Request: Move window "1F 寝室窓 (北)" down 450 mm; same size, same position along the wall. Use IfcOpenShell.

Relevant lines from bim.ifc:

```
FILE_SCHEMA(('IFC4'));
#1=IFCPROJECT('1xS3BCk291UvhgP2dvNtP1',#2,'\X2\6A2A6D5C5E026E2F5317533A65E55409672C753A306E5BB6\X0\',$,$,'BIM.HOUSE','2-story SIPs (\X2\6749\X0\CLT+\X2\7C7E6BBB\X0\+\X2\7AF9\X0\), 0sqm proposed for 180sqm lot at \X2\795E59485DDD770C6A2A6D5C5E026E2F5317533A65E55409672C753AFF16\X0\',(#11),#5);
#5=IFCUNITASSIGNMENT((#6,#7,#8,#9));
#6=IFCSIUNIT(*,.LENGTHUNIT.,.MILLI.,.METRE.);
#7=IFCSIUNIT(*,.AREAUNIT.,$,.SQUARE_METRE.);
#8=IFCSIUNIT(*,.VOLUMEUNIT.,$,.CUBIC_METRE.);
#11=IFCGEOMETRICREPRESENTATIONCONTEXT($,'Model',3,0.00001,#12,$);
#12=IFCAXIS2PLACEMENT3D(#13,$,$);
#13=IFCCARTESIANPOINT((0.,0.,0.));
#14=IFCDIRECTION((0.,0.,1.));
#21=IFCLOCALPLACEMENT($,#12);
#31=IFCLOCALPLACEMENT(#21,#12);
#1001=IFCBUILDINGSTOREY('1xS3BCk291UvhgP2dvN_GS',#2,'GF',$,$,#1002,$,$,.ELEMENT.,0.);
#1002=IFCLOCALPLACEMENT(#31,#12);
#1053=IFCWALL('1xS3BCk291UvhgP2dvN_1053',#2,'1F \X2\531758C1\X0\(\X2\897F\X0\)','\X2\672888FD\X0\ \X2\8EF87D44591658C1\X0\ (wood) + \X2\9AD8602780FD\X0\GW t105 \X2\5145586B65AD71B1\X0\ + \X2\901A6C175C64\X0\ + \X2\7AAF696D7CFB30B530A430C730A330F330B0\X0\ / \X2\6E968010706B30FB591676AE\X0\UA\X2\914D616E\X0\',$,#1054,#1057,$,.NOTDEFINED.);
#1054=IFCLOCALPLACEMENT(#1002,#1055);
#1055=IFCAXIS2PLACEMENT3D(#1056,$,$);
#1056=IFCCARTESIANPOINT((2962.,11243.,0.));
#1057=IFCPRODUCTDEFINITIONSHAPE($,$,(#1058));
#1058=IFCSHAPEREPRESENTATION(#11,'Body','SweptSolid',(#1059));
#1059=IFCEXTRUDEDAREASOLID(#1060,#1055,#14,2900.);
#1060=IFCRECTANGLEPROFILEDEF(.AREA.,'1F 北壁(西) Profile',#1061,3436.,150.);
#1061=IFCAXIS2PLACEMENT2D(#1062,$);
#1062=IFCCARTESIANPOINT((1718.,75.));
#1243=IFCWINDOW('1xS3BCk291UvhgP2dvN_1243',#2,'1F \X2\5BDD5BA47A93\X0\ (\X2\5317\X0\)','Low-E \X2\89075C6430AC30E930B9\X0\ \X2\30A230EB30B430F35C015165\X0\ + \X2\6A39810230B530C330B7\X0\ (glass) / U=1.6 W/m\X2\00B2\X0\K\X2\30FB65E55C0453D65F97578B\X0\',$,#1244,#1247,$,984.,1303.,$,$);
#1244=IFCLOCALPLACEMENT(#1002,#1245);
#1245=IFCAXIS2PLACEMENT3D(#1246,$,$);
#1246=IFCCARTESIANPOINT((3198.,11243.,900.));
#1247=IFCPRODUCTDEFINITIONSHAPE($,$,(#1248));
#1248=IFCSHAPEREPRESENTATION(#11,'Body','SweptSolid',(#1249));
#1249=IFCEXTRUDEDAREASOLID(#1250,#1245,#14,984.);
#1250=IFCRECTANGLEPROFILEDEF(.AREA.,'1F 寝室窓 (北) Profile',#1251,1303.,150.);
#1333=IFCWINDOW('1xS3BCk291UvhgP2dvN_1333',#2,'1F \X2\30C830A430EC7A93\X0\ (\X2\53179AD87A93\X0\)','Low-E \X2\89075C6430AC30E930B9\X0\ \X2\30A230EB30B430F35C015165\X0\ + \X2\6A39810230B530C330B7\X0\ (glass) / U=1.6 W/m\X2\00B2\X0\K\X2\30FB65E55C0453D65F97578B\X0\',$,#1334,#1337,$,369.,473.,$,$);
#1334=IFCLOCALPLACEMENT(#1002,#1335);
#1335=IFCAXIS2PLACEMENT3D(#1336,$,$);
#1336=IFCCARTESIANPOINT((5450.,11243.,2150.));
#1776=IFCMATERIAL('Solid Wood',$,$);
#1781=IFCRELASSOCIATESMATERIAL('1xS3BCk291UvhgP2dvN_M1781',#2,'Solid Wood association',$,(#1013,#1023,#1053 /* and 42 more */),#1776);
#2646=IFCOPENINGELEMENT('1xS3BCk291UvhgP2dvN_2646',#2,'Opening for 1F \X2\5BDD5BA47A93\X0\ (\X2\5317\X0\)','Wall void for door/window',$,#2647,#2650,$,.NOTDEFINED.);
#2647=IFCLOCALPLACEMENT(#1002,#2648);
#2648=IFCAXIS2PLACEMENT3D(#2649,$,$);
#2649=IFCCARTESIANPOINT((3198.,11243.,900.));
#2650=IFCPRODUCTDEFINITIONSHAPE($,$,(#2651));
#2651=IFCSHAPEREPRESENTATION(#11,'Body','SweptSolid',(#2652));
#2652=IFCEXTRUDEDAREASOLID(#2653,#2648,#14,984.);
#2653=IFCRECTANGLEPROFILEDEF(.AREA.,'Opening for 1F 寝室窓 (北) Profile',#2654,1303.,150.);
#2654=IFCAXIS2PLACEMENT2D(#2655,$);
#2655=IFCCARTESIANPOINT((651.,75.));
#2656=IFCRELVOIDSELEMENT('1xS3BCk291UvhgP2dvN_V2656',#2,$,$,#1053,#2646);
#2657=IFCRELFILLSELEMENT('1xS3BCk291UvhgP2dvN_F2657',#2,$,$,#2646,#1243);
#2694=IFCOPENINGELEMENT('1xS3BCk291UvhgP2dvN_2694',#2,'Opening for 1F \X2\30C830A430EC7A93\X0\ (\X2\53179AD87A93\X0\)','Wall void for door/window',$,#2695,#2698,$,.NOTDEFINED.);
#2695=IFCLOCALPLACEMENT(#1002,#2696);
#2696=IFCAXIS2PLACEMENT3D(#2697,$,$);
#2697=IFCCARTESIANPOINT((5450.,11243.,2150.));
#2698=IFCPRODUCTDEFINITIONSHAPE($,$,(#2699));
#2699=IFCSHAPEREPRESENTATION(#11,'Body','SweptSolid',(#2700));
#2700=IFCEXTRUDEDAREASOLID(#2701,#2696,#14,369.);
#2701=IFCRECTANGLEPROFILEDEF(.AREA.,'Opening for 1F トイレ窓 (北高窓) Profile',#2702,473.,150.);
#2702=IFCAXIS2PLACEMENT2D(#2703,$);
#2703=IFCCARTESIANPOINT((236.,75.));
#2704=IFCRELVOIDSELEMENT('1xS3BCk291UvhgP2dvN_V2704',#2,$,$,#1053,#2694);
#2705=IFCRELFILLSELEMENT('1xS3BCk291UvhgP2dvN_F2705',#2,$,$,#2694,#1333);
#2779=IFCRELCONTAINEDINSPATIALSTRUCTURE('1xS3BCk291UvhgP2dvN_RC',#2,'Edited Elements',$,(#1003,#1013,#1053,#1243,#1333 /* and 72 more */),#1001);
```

```python
import numpy as np
import ifcopenshell
import ifcopenshell.api.geometry
import ifcopenshell.util.placement
import ifcopenshell.util.unit

model = ifcopenshell.open("bim.ifc")
unit_scale = ifcopenshell.util.unit.calculate_unit_scale(model)

window = model.by_guid("1xS3BCk291UvhgP2dvN_1243")
opening = window.FillsVoids[0].RelatingOpeningElement
dz = -450.0

shift = np.array([0.0, 0.0, dz])
# The window is not placed relative to its opening, so move both.
for product in (opening, window):
    matrix = ifcopenshell.util.placement.get_local_placement(product.ObjectPlacement)
    matrix[:3, 3] += shift
    ifcopenshell.api.geometry.edit_object_placement(model, product=product, matrix=matrix, is_si=False)

print(f"moved by {dz * unit_scale:+.3f} m")

model.write("bim-out.ifc")
```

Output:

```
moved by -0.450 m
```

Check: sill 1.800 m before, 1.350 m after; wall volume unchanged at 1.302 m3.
